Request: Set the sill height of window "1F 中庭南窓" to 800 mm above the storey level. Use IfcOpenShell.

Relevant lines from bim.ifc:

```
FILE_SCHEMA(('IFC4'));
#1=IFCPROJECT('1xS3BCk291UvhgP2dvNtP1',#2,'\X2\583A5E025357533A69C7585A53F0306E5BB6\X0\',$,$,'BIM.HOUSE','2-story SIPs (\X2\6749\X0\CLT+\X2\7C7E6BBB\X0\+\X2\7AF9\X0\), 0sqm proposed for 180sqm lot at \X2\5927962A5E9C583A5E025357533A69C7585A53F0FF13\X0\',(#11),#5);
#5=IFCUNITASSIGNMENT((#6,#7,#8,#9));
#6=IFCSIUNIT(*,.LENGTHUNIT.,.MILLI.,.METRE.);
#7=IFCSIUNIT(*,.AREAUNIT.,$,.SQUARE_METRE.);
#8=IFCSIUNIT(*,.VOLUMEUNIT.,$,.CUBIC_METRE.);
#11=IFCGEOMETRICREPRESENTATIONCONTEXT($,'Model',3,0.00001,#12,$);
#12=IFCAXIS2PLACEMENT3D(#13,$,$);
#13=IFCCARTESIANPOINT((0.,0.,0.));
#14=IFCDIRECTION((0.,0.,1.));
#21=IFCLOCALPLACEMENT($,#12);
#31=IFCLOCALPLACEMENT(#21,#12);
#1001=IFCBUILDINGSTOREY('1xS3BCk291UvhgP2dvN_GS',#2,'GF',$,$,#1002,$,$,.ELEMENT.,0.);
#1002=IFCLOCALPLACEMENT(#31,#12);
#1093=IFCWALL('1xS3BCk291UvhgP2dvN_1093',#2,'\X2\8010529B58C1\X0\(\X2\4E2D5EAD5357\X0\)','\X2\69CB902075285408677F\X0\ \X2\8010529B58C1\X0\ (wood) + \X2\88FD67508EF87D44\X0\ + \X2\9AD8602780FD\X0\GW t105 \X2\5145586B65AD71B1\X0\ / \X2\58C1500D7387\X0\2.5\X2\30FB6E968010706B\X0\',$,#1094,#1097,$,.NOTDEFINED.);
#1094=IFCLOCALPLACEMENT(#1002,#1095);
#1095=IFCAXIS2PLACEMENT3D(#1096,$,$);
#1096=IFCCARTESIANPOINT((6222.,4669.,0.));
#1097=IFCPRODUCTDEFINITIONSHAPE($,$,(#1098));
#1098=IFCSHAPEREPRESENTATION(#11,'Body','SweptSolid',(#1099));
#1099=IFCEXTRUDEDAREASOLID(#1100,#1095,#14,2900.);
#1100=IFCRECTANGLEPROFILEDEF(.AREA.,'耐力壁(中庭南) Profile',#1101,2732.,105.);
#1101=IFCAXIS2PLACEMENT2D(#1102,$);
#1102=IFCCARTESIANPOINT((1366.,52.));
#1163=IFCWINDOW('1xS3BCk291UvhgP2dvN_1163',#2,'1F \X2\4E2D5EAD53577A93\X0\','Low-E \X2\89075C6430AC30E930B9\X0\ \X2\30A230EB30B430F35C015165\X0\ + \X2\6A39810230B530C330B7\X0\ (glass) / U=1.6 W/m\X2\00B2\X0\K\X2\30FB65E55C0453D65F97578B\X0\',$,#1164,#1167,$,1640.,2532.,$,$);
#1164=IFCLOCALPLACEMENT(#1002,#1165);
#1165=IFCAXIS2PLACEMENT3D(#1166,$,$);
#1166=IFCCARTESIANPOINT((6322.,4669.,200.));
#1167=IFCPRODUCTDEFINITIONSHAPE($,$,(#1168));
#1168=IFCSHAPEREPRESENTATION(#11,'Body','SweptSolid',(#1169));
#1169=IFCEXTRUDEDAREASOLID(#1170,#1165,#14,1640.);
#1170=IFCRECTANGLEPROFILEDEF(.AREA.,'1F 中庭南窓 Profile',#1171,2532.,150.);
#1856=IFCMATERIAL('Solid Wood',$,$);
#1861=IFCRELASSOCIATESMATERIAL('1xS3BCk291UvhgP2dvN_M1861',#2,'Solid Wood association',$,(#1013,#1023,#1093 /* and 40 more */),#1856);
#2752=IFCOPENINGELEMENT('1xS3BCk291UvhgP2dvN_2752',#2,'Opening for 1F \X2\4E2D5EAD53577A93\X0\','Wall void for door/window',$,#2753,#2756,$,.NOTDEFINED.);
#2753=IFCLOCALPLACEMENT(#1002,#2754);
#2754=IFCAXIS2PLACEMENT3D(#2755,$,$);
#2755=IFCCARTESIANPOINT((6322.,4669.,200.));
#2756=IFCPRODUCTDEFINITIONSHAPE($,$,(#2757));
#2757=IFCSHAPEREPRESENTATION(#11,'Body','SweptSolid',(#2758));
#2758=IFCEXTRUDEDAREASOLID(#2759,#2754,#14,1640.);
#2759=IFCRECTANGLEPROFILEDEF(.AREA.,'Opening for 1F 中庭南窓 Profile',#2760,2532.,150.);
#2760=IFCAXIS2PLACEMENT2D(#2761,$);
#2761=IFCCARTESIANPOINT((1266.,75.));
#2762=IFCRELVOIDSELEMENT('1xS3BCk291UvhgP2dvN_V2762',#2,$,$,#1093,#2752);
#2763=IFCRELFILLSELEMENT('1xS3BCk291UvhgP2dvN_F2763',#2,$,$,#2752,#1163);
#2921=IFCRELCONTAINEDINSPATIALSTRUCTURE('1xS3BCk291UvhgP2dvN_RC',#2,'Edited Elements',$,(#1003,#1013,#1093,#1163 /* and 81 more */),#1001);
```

```python
import numpy as np
import ifcopenshell
import ifcopenshell.api.geometry
import ifcopenshell.geom
import ifcopenshell.util.element
import ifcopenshell.util.placement
import ifcopenshell.util.shape
import ifcopenshell.util.unit

model = ifcopenshell.open("bim.ifc")
unit_scale = ifcopenshell.util.unit.calculate_unit_scale(model)

window = model.by_guid("1xS3BCk291UvhgP2dvN_1163")
opening = window.FillsVoids[0].RelatingOpeningElement
storey = ifcopenshell.util.element.get_container(window, ifc_class="IfcBuildingStorey")
level = ifcopenshell.util.placement.get_local_placement(storey.ObjectPlacement)[2, 3]

# The opening's origin need not be at the sill, so measure its lowest point.
shape = ifcopenshell.geom.create_shape(ifcopenshell.geom.settings(), opening)
bottom = ifcopenshell.util.shape.get_shape_bottom_elevation(shape, shape.geometry) / unit_scale
dz = level + 0.8 / unit_scale - bottom

shift = np.array([0.0, 0.0, dz])
# The window is not placed relative to its opening, so move both.
for product in (opening, window):
    matrix = ifcopenshell.util.placement.get_local_placement(product.ObjectPlacement)
    matrix[:3, 3] += shift
    ifcopenshell.api.geometry.edit_object_placement(model, product=product, matrix=matrix, is_si=False)

print(f"moved by {dz * unit_scale:+.3f} m")

model.write("bim-out.ifc")
```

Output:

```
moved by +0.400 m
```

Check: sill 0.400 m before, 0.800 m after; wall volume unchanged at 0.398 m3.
